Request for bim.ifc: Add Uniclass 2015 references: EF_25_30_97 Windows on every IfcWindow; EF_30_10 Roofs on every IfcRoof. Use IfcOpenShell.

First a look at what the model holds.

```python
import ifcopenshell

model = ifcopenshell.open("bim.ifc")
print(model.schema)
print("classifications:", [c.Name for c in model.by_type("IfcClassification")])
for ifc_class in ("IfcDoor", "IfcRoof", "IfcStair", "IfcWall", "IfcWindow"):
    print(ifc_class, len(model.by_type(ifc_class)))
```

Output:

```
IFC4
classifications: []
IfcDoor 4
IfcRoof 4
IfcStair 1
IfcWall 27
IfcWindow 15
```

```python
import ifcopenshell
import ifcopenshell.api.classification

model = ifcopenshell.open("bim.ifc")

system = ifcopenshell.api.classification.add_classification(model, classification="Uniclass 2015")

codes = {
    "IfcWindow": ("EF_25_30_97", "Windows"),
    "IfcRoof": ("EF_30_10", "Roofs"),
}
for ifc_class, (code, name) in codes.items():
    products = model.by_type(ifc_class)
    ifcopenshell.api.classification.add_reference(
        model, products=products, classification=system, identification=code, name=name
    )
    print(code, len(products))

model.write("bim_rev.ifc")
```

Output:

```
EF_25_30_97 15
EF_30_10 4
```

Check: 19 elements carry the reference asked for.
